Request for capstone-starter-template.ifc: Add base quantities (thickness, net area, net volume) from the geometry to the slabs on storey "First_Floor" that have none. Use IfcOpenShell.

First a look at what the model holds.

```python
import ifcopenshell
import ifcopenshell.util.element
import ifcopenshell.util.unit

model = ifcopenshell.open("capstone-starter-template.ifc")
print(model.schema)
for unit_type in ("LENGTHUNIT", "AREAUNIT", "VOLUMEUNIT"):
    print(unit_type, ifcopenshell.util.unit.calculate_unit_scale(model, unit_type))
storey = next(s for s in model.by_type("IfcBuildingStorey") if s.Name == "First_Floor")
slabs = [e for e in ifcopenshell.util.element.get_decomposition(storey) if e.is_a("IfcSlab")]
for e in sorted(slabs, key=lambda e: e.id()):
    print(e.id(), e.is_a(), e.Name, list(ifcopenshell.util.element.get_psets(e, qtos_only=True)), sep=" | ")
```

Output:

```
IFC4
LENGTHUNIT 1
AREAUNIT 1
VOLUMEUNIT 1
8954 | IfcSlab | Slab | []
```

```python
import ifcopenshell
import ifcopenshell.api.pset
import ifcopenshell.geom
import ifcopenshell.util.element
import ifcopenshell.util.shape
import ifcopenshell.util.unit

model = ifcopenshell.open("capstone-starter-template.ifc")
unit_scale = ifcopenshell.util.unit.calculate_unit_scale(model)
area_scale = ifcopenshell.util.unit.calculate_unit_scale(model, "AREAUNIT")
volume_scale = ifcopenshell.util.unit.calculate_unit_scale(model, "VOLUMEUNIT")
settings = ifcopenshell.geom.settings()

storey = next(s for s in model.by_type("IfcBuildingStorey") if s.Name == "First_Floor")
slabs = [e for e in ifcopenshell.util.element.get_decomposition(storey) if e.is_a("IfcSlab")]

for e in sorted(slabs, key=lambda e: e.id()):
    if ifcopenshell.util.element.get_psets(e, qtos_only=True, should_inherit=False):
        continue
    # Geometry comes back in metres, in the element's own axes.
    shape = ifcopenshell.geom.create_shape(settings, e)
    values = {
        "Width": ifcopenshell.util.shape.get_z(shape.geometry) / unit_scale,
        "NetArea": ifcopenshell.util.shape.get_footprint_area(shape.geometry) / area_scale,
        "NetVolume": ifcopenshell.util.shape.get_volume(shape.geometry) / volume_scale,
    }
    qto = ifcopenshell.api.pset.add_qto(model, product=e, name="Qto_SlabBaseQuantities")
    ifcopenshell.api.pset.edit_qto(model, qto=qto, properties=values)
    print(e.id(), {k: round(v, 3) for k, v in values.items()})

model.write("capstone-starter-template_updated.ifc")
```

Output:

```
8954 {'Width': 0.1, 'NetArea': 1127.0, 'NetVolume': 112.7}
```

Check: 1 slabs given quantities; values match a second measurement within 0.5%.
